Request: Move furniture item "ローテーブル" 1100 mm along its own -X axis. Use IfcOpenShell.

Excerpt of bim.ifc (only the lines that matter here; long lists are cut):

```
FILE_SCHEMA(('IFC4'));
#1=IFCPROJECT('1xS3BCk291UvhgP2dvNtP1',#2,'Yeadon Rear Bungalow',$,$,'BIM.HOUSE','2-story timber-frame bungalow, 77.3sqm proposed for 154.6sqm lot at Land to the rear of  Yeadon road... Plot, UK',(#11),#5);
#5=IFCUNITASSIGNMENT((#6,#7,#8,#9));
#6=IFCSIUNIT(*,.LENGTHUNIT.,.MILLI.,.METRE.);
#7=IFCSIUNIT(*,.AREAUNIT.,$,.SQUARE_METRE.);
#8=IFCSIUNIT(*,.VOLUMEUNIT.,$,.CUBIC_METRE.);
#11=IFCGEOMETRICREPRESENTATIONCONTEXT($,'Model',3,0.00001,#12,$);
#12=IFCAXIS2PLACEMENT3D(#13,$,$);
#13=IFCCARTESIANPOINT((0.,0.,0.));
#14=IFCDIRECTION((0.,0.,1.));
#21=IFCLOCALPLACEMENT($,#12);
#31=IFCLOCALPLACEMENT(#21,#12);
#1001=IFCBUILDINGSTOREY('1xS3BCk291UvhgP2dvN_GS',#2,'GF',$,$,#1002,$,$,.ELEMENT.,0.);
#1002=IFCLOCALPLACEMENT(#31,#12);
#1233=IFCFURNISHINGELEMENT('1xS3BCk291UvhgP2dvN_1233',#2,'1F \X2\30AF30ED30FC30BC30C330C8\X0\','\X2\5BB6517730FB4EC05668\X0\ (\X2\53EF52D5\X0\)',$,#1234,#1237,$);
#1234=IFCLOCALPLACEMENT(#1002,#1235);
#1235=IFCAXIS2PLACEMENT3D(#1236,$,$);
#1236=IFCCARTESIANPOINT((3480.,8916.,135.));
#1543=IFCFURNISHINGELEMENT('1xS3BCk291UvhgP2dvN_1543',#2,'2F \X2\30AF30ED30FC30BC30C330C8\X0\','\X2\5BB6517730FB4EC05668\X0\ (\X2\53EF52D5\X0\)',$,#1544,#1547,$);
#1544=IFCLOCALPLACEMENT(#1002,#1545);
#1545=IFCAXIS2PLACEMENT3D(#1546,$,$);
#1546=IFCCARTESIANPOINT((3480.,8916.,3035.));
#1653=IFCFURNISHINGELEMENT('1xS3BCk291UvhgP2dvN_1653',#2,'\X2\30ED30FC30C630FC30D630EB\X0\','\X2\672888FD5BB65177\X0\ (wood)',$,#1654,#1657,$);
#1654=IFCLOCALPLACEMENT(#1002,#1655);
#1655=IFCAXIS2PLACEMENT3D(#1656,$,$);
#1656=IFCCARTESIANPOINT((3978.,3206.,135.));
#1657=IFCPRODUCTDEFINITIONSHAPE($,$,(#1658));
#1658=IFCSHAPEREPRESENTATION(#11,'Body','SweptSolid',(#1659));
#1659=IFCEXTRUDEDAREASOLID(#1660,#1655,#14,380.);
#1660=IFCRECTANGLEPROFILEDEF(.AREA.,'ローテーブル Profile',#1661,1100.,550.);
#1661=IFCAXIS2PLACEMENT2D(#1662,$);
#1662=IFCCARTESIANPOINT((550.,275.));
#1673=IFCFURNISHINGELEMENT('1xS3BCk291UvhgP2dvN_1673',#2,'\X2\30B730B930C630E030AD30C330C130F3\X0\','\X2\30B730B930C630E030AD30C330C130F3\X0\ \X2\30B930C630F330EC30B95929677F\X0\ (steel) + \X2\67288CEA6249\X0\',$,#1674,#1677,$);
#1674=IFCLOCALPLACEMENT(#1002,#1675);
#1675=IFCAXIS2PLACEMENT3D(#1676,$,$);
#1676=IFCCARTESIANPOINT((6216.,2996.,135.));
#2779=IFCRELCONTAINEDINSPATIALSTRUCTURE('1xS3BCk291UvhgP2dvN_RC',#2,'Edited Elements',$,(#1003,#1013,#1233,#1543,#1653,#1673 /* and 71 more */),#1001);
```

```python
import ifcopenshell
import ifcopenshell.api.geometry
import ifcopenshell.util.placement
import ifcopenshell.util.unit

model = ifcopenshell.open("bim.ifc")
unit_scale = ifcopenshell.util.unit.calculate_unit_scale(model)

item = model.by_id(1653)
matrix = ifcopenshell.util.placement.get_local_placement(item.ObjectPlacement)
matrix[:3, 3] -= matrix[:3, 0] * 1.1 / unit_scale
ifcopenshell.api.geometry.edit_object_placement(model, product=item, matrix=matrix, is_si=False)

print(ifcopenshell.util.placement.get_local_placement(item.ObjectPlacement).round(3) + 0.0)

model.write("bim_edited.ifc")
```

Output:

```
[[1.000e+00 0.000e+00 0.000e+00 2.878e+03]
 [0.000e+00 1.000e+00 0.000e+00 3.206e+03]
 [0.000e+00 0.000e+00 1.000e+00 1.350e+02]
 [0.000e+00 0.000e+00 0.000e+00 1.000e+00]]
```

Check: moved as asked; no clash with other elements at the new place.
